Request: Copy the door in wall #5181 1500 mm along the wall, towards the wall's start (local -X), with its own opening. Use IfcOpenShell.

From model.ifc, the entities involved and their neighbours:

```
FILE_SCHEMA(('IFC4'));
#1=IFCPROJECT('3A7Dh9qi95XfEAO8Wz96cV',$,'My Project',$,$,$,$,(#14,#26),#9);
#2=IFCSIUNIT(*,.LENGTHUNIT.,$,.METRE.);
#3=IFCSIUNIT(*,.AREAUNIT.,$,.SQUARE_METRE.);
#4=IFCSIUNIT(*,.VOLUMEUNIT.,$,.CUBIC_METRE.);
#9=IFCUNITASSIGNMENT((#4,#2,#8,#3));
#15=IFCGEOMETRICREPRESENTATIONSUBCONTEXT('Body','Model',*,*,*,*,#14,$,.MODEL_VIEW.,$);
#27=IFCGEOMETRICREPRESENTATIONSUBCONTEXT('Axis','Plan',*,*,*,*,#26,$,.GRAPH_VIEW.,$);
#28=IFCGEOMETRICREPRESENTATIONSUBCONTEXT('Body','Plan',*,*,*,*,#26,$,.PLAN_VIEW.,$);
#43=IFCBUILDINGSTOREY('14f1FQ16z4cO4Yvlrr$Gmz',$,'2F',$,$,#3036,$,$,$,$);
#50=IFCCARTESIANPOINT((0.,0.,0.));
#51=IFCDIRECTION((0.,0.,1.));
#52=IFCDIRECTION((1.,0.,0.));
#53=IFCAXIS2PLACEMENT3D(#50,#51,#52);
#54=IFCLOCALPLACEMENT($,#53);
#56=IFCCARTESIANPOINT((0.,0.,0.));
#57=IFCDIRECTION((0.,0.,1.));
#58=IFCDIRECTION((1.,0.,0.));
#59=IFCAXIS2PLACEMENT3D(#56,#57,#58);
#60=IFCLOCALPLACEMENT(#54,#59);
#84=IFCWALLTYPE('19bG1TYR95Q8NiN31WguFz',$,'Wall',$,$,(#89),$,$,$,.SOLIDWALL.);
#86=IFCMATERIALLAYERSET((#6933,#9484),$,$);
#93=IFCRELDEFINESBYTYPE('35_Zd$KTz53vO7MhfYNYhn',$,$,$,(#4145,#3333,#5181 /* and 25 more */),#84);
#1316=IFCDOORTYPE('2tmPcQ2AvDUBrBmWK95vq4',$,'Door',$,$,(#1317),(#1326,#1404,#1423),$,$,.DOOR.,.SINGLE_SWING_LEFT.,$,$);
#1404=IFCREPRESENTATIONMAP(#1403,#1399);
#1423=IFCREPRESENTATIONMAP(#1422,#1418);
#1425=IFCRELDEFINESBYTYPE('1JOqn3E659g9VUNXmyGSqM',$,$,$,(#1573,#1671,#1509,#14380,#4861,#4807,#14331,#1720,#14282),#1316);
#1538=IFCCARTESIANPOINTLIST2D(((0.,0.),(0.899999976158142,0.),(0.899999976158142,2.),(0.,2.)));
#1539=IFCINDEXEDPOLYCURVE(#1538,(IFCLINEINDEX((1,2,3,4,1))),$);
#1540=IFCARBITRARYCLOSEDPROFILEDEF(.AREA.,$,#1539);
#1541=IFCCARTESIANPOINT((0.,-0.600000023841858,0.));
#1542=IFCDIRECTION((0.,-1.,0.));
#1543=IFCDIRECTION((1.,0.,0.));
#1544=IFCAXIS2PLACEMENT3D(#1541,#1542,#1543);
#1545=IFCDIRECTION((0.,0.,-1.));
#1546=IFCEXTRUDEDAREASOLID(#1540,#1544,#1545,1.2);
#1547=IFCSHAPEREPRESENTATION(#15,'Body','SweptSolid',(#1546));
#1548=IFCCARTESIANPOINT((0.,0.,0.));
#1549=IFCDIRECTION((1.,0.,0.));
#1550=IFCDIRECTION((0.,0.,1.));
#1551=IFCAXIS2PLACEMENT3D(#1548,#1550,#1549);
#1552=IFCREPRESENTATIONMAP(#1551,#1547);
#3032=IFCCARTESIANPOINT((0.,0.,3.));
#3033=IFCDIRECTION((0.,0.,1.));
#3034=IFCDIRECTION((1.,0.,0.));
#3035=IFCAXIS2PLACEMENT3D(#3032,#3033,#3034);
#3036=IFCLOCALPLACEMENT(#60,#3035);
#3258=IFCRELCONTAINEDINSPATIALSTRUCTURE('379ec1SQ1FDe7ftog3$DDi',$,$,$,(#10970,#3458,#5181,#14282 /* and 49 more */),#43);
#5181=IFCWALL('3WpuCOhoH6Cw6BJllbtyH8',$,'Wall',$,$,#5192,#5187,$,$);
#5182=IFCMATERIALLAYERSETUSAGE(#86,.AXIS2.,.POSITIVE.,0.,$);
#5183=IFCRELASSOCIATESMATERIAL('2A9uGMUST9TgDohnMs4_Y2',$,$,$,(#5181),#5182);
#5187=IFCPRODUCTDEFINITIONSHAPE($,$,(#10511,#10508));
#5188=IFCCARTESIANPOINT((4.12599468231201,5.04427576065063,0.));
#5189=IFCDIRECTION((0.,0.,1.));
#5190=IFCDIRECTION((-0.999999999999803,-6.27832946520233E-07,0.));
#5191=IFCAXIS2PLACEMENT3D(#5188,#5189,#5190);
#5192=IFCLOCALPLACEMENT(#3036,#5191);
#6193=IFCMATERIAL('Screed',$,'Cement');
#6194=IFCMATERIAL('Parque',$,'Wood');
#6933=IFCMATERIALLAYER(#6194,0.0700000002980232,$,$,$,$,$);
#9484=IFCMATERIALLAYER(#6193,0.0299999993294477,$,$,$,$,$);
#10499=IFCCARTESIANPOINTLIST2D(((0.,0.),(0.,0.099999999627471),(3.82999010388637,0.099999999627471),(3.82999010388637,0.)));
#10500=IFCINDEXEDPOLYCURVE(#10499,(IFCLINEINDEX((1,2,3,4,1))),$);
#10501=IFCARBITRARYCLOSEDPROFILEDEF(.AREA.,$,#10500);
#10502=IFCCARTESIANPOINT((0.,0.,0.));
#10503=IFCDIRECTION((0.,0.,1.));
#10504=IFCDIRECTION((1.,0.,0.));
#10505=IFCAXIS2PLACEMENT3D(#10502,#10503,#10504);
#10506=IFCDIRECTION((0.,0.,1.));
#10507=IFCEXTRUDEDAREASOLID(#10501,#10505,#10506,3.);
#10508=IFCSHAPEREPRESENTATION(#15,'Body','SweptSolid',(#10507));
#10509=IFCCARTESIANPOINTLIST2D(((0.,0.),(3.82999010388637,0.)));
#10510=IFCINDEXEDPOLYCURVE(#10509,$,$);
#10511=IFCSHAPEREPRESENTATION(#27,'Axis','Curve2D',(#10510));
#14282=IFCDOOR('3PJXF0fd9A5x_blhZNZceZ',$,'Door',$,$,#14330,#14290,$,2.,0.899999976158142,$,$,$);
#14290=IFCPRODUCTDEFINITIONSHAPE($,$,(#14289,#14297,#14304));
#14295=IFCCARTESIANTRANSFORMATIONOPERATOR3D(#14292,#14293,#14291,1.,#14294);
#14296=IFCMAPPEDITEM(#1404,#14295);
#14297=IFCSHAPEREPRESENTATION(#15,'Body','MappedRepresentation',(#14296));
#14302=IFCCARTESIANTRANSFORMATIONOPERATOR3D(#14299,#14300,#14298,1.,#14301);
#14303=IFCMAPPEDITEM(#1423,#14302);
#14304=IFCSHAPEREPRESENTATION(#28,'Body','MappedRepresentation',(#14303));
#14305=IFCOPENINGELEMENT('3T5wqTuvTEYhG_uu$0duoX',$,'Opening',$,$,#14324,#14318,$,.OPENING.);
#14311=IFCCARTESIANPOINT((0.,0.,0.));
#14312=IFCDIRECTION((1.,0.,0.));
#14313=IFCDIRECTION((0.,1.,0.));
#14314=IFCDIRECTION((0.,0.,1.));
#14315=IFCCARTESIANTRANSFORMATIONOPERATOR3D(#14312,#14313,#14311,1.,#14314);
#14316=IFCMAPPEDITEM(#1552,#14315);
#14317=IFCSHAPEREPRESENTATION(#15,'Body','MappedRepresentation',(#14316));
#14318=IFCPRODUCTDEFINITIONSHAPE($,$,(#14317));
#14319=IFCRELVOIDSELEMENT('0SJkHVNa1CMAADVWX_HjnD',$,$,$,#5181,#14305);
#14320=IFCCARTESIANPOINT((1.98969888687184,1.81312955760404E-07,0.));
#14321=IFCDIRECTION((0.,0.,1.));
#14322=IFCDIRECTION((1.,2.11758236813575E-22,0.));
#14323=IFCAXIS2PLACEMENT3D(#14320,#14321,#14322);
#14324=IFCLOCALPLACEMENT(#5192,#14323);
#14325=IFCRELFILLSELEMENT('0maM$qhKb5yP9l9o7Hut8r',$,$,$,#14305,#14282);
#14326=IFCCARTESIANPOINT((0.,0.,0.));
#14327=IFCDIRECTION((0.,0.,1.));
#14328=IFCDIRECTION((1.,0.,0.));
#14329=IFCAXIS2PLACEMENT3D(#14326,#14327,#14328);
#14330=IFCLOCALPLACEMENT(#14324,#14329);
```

```python
import ifcopenshell
import ifcopenshell.api.feature
import ifcopenshell.api.geometry
import ifcopenshell.api.root
import ifcopenshell.geom
import ifcopenshell.util.element
import ifcopenshell.util.placement
import ifcopenshell.util.shape
import ifcopenshell.util.unit

model = ifcopenshell.open("model.ifc")
unit_scale = ifcopenshell.util.unit.calculate_unit_scale(model)
settings = ifcopenshell.geom.settings()


def volume(element):
    """Net volume in cubic metres, openings subtracted."""
    shape = ifcopenshell.geom.create_shape(settings, element)
    return ifcopenshell.util.shape.get_volume(shape.geometry)


door = model.by_guid("3PJXF0fd9A5x_blhZNZceZ")
opening = door.FillsVoids[0].RelatingOpeningElement
wall = opening.VoidsElements[0].RelatingBuildingElement
before = volume(wall)
shift = ifcopenshell.util.placement.get_local_placement(wall.ObjectPlacement)[:3, 0] * -1.5 / unit_scale

# copy_class copies the void relationship, type, container and properties, but no geometry.
new_opening = ifcopenshell.api.root.copy_class(model, product=opening)
new_opening.Representation = ifcopenshell.util.element.copy_deep(
    model, opening.Representation, exclude=["IfcGeometricRepresentationContext", "IfcRepresentationMap"]
)
new_door = ifcopenshell.api.root.copy_class(model, product=door)
new_door.Representation = ifcopenshell.util.element.copy_deep(
    model, door.Representation, exclude=["IfcGeometricRepresentationContext", "IfcRepresentationMap"]
)
ifcopenshell.api.feature.add_filling(model, opening=new_opening, element=new_door)

for old, new in ((opening, new_opening), (door, new_door)):
    matrix = ifcopenshell.util.placement.get_local_placement(old.ObjectPlacement)
    matrix[:3, 3] += shift
    ifcopenshell.api.geometry.edit_object_placement(model, product=new, matrix=matrix, is_si=False)

after = volume(wall)

print(f"wall volume {before:.3f} -> {after:.3f} m3")

model.write("model_v2.ifc")
```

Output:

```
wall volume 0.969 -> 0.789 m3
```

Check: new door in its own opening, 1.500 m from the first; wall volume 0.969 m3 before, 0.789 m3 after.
